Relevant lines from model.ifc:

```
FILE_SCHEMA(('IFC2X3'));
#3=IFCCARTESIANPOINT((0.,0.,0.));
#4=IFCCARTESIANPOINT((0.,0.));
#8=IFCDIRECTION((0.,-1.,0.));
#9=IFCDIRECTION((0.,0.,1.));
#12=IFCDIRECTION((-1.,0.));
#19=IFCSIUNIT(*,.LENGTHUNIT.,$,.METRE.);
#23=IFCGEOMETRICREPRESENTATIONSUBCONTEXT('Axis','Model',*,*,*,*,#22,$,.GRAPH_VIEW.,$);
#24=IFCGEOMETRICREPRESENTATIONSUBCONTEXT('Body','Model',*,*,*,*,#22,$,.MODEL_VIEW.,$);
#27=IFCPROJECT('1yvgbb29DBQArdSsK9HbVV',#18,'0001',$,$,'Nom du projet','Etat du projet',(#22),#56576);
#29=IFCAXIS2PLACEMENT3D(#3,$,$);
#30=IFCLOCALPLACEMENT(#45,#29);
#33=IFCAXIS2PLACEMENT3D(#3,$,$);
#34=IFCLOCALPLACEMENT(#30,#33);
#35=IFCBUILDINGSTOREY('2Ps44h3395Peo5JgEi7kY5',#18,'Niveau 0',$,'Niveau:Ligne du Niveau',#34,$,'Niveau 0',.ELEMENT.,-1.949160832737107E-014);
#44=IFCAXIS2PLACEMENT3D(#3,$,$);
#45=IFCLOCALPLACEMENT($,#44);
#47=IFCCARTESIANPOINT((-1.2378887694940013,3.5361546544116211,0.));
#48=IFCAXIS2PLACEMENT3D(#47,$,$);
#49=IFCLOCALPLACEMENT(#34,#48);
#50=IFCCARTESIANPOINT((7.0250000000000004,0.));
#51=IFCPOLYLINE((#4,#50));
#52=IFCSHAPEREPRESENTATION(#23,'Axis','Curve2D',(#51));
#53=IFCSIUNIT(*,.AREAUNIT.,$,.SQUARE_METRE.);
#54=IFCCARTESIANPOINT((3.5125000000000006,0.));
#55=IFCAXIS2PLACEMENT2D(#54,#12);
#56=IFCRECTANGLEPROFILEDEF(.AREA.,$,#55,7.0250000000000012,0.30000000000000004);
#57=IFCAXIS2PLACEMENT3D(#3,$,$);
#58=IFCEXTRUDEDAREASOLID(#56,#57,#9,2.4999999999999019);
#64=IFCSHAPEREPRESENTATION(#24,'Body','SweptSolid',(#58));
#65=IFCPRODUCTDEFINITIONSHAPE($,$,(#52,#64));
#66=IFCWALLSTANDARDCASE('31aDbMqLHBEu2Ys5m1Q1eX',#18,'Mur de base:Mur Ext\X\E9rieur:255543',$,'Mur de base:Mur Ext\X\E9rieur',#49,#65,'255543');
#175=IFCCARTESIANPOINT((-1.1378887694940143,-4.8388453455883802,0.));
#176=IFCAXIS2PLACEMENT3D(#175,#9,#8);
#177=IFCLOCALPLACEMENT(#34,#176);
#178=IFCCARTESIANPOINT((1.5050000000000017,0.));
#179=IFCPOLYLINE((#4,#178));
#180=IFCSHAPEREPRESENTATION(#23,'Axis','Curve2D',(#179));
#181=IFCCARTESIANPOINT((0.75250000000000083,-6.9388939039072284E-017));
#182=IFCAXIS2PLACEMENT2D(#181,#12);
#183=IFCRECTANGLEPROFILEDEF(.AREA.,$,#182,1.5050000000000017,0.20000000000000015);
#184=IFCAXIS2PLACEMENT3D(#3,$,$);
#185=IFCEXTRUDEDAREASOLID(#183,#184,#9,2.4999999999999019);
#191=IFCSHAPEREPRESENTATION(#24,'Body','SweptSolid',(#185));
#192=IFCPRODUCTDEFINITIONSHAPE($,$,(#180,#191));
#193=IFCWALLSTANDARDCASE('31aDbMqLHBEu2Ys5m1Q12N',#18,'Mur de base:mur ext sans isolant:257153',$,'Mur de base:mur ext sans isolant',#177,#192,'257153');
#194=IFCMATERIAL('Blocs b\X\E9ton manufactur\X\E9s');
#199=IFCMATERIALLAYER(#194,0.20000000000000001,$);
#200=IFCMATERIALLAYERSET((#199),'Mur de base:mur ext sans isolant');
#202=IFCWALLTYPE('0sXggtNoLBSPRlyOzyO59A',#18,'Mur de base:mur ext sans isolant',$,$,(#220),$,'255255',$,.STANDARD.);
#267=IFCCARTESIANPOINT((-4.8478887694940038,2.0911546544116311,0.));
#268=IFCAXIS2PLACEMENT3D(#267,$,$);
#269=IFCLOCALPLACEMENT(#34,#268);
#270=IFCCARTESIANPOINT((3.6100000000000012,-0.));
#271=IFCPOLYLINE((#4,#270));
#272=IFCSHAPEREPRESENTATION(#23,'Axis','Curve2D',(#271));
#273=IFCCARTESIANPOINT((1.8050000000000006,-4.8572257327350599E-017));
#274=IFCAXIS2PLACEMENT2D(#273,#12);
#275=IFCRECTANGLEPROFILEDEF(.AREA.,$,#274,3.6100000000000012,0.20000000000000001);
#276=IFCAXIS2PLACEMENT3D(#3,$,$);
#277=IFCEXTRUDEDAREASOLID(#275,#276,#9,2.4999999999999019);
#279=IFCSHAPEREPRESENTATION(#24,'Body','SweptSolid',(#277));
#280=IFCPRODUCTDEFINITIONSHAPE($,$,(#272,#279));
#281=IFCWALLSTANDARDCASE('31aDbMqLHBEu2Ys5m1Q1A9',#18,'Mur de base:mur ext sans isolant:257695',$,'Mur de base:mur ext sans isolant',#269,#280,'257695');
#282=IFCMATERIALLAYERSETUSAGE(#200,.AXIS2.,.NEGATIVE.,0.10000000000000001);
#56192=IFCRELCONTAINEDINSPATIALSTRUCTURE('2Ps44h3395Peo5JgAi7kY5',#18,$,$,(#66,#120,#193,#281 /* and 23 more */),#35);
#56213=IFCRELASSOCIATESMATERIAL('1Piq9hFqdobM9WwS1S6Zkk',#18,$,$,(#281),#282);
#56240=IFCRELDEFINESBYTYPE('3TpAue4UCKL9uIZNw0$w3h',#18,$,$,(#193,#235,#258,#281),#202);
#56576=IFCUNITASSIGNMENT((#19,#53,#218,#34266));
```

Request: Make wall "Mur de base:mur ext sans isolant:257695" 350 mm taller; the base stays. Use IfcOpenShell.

```python
import ifcopenshell
import ifcopenshell.geom
import ifcopenshell.util.representation
import ifcopenshell.util.shape
import ifcopenshell.util.unit

model = ifcopenshell.open("model.ifc")
unit_scale = ifcopenshell.util.unit.calculate_unit_scale(model)
settings = ifcopenshell.geom.settings()


def volume(element):
    """Net volume in cubic metres, openings subtracted."""
    shape = ifcopenshell.geom.create_shape(settings, element)
    return ifcopenshell.util.shape.get_volume(shape.geometry)


wall = model.by_guid("31aDbMqLHBEu2Ys5m1Q1A9")
before = volume(wall)

body = ifcopenshell.util.representation.get_representation(wall, "Model", "Body")
solid = body.Items[0]
old_height = solid.Depth
solid.Depth += 0.35 / unit_scale
after = volume(wall)

print(f"height {old_height:g} -> {solid.Depth:g}, volume {before:.3f} -> {after:.3f} m3")

model.write("model_rev.ifc")
```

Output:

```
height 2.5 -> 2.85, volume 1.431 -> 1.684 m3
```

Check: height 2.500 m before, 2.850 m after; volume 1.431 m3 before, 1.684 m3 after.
